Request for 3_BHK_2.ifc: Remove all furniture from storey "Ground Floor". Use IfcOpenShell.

First a look at what the model holds.

```python
import ifcopenshell
import ifcopenshell.util.element

model = ifcopenshell.open("3_BHK_2.ifc")
print(model.schema)
storey = next(s for s in model.by_type("IfcBuildingStorey") if s.Name == "Ground Floor")
furniture = [e for e in ifcopenshell.util.element.get_decomposition(storey) if e.is_a("IfcFurnishingElement")]
seen = {}
for e in furniture:
    element_type = ifcopenshell.util.element.get_type(e)
    name = element_type.Name if element_type not in (None, e) else None
    seen[name] = seen.get(name, 0) + 1
for name, count in sorted(seen.items(), key=str):
    print(count, "x", name)
```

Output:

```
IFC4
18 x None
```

```python
import ifcopenshell
import ifcopenshell.api.root
import ifcopenshell.util.element

model = ifcopenshell.open("3_BHK_2.ifc")

storey = next(s for s in model.by_type("IfcBuildingStorey") if s.Name == "Ground Floor")
furniture = [e for e in ifcopenshell.util.element.get_decomposition(storey) if e.is_a("IfcFurnishingElement")]

for e in furniture:
    ifcopenshell.api.root.remove_product(model, product=e)
print(len(furniture), "removed")

model.write("3_BHK_2-out.ifc")
```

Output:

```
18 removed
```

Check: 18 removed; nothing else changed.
